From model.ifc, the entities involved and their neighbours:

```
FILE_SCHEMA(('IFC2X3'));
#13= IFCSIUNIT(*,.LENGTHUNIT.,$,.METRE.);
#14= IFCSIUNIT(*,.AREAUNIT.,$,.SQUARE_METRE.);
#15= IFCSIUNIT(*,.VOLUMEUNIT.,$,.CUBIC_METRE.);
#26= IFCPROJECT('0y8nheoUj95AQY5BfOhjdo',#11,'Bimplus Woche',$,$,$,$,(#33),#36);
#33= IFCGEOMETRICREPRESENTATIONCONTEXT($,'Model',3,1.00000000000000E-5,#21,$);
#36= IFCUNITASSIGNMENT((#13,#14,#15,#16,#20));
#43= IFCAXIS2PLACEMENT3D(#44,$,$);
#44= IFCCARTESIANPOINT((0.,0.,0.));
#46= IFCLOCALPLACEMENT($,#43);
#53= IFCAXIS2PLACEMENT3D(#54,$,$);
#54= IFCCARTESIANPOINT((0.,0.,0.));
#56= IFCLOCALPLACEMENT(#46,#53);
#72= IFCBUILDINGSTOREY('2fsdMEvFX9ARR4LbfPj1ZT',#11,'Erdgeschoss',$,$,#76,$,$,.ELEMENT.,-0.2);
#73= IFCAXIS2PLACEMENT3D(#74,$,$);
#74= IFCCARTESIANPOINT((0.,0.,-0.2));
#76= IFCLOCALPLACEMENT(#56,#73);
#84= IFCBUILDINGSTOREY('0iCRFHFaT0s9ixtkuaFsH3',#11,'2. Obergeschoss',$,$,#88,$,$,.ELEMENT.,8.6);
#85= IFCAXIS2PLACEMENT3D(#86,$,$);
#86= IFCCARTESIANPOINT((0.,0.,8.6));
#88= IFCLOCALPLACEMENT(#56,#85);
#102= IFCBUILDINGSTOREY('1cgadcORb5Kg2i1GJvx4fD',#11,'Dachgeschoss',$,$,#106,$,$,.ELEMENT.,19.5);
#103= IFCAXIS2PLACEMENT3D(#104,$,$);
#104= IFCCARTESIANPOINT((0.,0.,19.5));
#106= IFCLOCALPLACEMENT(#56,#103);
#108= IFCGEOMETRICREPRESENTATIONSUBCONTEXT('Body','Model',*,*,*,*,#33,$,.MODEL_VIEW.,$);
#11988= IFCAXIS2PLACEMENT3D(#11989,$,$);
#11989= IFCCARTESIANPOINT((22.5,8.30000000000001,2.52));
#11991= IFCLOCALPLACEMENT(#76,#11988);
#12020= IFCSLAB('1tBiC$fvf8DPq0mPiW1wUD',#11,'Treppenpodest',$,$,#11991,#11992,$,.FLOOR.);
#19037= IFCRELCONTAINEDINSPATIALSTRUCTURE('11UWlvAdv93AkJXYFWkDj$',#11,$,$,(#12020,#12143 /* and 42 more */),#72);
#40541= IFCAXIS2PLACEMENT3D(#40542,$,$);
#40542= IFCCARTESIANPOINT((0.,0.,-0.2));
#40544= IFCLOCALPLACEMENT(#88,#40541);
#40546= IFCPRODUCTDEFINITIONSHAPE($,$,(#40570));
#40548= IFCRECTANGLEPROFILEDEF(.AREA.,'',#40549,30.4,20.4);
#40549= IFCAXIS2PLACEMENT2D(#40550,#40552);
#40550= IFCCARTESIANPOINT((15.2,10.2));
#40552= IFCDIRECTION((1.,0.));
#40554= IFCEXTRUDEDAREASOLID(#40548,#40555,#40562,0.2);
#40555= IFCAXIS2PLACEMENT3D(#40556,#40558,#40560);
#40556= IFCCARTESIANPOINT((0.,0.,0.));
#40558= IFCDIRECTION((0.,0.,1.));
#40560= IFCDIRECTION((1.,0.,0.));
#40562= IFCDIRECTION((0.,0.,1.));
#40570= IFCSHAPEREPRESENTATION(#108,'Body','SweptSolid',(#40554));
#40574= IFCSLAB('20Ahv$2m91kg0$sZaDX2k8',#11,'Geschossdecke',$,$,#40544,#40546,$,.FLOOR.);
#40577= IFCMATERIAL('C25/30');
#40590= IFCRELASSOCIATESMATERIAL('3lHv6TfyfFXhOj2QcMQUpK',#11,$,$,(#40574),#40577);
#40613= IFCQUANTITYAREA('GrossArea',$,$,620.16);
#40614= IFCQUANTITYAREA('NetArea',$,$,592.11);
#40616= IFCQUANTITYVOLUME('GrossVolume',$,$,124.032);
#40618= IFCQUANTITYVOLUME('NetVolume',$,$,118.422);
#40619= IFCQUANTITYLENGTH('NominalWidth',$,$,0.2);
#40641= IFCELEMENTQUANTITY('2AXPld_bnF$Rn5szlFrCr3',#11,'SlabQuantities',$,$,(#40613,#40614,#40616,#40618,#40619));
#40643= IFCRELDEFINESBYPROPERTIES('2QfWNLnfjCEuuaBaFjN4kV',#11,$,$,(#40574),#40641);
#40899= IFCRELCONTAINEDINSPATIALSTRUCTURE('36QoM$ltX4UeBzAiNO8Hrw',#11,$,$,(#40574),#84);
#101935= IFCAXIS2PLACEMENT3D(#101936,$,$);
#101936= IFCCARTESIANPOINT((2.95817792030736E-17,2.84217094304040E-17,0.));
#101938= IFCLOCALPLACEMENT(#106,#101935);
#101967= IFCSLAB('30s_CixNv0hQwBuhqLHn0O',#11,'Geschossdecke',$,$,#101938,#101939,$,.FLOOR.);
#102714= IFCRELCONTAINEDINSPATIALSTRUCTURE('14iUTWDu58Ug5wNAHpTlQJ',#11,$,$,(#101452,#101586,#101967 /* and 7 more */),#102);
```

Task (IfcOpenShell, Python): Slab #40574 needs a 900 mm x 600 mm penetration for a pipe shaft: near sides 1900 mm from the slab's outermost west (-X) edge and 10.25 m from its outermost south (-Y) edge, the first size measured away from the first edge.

```python
import numpy as np
import ifcopenshell
import ifcopenshell.api.feature
import ifcopenshell.api.geometry
import ifcopenshell.api.pset
import ifcopenshell.api.root
import ifcopenshell.geom
import ifcopenshell.util.element
import ifcopenshell.util.placement
import ifcopenshell.util.representation
import ifcopenshell.util.shape
import ifcopenshell.util.unit

model = ifcopenshell.open("model.ifc")
unit_scale = ifcopenshell.util.unit.calculate_unit_scale(model)
area_scale = ifcopenshell.util.unit.calculate_unit_scale(model, "AREAUNIT")
volume_scale = ifcopenshell.util.unit.calculate_unit_scale(model, "VOLUMEUNIT")
settings = ifcopenshell.geom.settings()


def volume(element):
    """Net volume in cubic metres, openings subtracted."""
    shape = ifcopenshell.geom.create_shape(settings, element)
    return ifcopenshell.util.shape.get_volume(shape.geometry)


slab = model.by_guid("20Ahv$2m91kg0$sZaDX2k8")
before = volume(slab)

# Extent in the slab's own axes, in metres. The edges named are its -X and -Y sides.
slab_shape = ifcopenshell.geom.create_shape(settings, slab)
vertices = ifcopenshell.util.shape.get_vertices(slab_shape.geometry)
x_min, y_min, bottom = vertices.min(axis=0)
top = vertices[:, 2].max()

opening = ifcopenshell.api.root.create_entity(model, ifc_class="IfcOpeningElement", name="Pipe shaft opening")
context = ifcopenshell.util.representation.get_context(model, "Model", "Body", "MODEL_VIEW")
width, depth = 0.9, 0.6
outline = [(0.0, 0.0), (width, 0.0), (width, depth), (0.0, depth), (0.0, 0.0)]
# Overshoot both faces by 50 mm so the cut is clean.
shape = ifcopenshell.api.geometry.add_slab_representation(
    model, context=context, depth=top - bottom + 0.1, polyline=outline
)
ifcopenshell.api.geometry.assign_representation(model, product=opening, representation=shape)

matrix = ifcopenshell.util.placement.get_local_placement(slab.ObjectPlacement)
matrix[:, 3] = matrix @ np.append(np.array([x_min + 1.9, y_min + 10.25, bottom - 0.05]) / unit_scale, 1.0)
ifcopenshell.api.geometry.edit_object_placement(model, product=opening, matrix=matrix, is_si=False)
ifcopenshell.api.feature.add_feature(model, feature=opening, element=slab)

after = volume(slab)

# Update the slab's stored quantities.
qto = model.by_id(ifcopenshell.util.element.get_pset(slab, "SlabQuantities", should_inherit=False)["id"])
ifcopenshell.api.pset.edit_qto(model, qto=qto, properties={
    "NetArea": after / (top - bottom) / area_scale,
    "NetVolume": after / volume_scale,
})

print(f"slab volume {before:.3f} -> {after:.3f} m3")

model.write("model_edited.ifc")
```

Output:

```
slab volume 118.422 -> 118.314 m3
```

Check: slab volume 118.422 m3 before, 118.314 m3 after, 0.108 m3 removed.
